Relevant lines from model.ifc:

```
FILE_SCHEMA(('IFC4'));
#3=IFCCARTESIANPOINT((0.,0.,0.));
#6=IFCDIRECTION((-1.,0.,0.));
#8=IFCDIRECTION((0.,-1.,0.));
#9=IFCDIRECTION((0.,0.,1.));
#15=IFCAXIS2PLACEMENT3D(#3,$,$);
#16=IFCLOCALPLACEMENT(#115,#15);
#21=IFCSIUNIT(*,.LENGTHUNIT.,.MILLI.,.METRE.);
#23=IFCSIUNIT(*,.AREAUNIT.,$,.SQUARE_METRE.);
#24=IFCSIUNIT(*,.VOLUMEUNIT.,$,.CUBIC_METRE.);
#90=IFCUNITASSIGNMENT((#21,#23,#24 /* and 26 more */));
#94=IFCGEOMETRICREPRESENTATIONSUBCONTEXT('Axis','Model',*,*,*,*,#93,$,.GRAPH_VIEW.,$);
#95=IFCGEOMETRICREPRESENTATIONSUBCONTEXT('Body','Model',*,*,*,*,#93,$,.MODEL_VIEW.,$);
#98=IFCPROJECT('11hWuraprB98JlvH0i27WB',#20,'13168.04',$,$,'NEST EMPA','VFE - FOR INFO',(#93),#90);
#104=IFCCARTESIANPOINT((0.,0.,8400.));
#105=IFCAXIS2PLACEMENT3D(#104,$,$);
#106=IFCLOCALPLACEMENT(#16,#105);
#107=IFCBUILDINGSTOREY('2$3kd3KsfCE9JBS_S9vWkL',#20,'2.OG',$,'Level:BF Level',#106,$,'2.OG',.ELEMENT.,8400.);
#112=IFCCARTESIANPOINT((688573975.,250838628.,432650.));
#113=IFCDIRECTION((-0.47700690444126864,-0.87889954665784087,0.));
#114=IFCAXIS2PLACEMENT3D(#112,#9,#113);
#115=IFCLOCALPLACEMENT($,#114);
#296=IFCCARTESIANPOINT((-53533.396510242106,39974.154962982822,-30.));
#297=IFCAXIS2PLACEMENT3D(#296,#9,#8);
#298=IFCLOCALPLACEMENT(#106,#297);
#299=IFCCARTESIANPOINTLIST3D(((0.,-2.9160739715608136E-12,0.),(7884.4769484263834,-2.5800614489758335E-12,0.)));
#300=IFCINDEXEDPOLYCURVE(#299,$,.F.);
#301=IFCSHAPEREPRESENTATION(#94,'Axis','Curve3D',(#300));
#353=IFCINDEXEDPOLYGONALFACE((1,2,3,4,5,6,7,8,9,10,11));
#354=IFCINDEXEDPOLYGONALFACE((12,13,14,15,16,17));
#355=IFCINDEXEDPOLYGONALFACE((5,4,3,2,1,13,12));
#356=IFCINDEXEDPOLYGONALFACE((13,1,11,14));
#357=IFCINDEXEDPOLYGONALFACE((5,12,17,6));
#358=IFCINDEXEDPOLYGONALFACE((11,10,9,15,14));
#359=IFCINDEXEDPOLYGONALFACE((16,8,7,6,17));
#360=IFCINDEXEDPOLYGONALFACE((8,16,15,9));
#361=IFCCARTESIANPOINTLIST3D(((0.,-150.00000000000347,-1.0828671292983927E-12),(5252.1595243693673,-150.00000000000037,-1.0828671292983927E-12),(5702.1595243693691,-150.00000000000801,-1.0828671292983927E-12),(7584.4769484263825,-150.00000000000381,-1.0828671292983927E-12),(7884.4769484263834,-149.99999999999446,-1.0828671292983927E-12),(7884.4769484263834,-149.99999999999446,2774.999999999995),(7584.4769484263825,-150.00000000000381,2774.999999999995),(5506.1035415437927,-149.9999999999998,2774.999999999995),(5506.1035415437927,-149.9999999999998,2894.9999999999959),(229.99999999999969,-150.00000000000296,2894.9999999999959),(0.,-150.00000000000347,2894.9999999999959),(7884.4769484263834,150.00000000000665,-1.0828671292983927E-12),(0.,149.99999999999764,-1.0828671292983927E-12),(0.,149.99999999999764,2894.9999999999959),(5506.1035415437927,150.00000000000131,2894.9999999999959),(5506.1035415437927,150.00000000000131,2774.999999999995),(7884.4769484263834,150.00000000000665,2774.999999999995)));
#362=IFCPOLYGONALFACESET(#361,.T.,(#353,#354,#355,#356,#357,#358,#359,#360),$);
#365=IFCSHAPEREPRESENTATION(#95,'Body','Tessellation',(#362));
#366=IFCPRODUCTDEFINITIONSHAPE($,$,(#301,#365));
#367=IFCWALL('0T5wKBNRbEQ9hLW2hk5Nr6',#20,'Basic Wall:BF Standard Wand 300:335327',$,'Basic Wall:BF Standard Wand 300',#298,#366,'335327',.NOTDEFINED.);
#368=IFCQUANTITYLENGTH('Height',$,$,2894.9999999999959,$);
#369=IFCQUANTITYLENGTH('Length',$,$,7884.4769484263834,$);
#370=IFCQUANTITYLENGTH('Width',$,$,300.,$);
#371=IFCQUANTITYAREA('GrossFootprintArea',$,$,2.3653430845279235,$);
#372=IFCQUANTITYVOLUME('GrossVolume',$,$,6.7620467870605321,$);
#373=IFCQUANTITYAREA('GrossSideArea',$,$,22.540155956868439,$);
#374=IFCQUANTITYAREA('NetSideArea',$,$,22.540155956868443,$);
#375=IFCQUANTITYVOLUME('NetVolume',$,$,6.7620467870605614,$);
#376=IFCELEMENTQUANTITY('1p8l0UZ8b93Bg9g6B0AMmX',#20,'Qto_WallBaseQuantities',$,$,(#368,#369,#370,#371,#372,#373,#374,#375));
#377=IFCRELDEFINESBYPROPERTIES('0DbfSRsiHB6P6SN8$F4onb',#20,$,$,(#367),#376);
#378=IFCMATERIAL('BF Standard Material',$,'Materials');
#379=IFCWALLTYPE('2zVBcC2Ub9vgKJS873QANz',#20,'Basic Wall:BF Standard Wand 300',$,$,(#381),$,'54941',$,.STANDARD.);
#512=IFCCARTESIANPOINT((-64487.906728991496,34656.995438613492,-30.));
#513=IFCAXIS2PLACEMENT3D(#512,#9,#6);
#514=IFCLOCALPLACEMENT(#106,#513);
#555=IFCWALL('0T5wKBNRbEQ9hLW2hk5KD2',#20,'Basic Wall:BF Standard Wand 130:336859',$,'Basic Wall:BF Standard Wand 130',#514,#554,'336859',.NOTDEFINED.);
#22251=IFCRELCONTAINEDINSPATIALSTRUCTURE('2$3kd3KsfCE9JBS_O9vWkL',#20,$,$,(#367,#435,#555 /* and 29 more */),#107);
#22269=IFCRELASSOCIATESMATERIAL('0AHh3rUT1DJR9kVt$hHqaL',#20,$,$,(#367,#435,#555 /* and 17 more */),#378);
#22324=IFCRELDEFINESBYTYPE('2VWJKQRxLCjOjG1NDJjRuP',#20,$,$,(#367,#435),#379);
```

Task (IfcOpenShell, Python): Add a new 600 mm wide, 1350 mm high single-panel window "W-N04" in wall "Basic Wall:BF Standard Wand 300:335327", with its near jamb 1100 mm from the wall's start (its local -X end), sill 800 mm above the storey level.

```python
import numpy as np
import ifcopenshell
import ifcopenshell.api.feature
import ifcopenshell.api.geometry
import ifcopenshell.api.pset
import ifcopenshell.api.root
import ifcopenshell.api.spatial
import ifcopenshell.geom
import ifcopenshell.util.element
import ifcopenshell.util.placement
import ifcopenshell.util.representation
import ifcopenshell.util.shape
import ifcopenshell.util.unit

model = ifcopenshell.open("model.ifc")
unit_scale = ifcopenshell.util.unit.calculate_unit_scale(model)
area_scale = ifcopenshell.util.unit.calculate_unit_scale(model, "AREAUNIT")
volume_scale = ifcopenshell.util.unit.calculate_unit_scale(model, "VOLUMEUNIT")
settings = ifcopenshell.geom.settings()


def volume(element):
    """Net volume in cubic metres, openings subtracted."""
    shape = ifcopenshell.geom.create_shape(settings, element)
    return ifcopenshell.util.shape.get_volume(shape.geometry)


wall = model.by_guid("0T5wKBNRbEQ9hLW2hk5Nr6")
storey = ifcopenshell.util.element.get_container(wall, ifc_class="IfcBuildingStorey")
context = ifcopenshell.util.representation.get_context(model, "Model", "Body", "MODEL_VIEW")
before = volume(wall)

width, height, from_end, sill = 0.6, 1.35, 1.1, 0.8  # metres

# The wall runs along its own X axis, and the end named is its -X end.
wall_shape = ifcopenshell.geom.create_shape(settings, wall)
x, y, z = ifcopenshell.util.shape.get_vertices(wall_shape.geometry).T
start = x.min() + from_end
face, thickness = float(y.min()), float(y.max() - y.min())
wall_matrix = ifcopenshell.util.placement.get_local_placement(wall.ObjectPlacement)
level = ifcopenshell.util.placement.get_local_placement(storey.ObjectPlacement)[2, 3]


def in_wall(x, y):
    """Placement at x, y metres in the wall's axes, at sill height."""
    matrix = wall_matrix.copy()
    matrix[:, 3] = wall_matrix @ np.array([x / unit_scale, y / unit_scale, 0.0, 1.0])
    matrix[2, 3] = level + sill / unit_scale
    return matrix


# Opening: a box that overshoots both wall faces by 50 mm.
opening = ifcopenshell.api.root.create_entity(model, ifc_class="IfcOpeningElement", predefined_type="OPENING")
box = ifcopenshell.api.geometry.add_wall_representation(
    model, context=context, length=width, height=height, thickness=thickness + 0.1
)
ifcopenshell.api.geometry.assign_representation(model, product=opening, representation=box)
ifcopenshell.api.geometry.edit_object_placement(model, product=opening, matrix=in_wall(start, face - 0.05), is_si=False)
ifcopenshell.api.feature.add_feature(model, feature=opening, element=wall)

window = ifcopenshell.api.root.create_entity(model, ifc_class="IfcWindow", name="W-N04", predefined_type="WINDOW")
window.OverallWidth, window.OverallHeight = width / unit_scale, height / unit_scale
window.PartitioningType = "SINGLE_PANEL"
body = ifcopenshell.api.geometry.add_window_representation(
    model,
    context=context,
    overall_width=window.OverallWidth,
    overall_height=window.OverallHeight,
    partition_type="SINGLE_PANEL",
)
ifcopenshell.api.geometry.assign_representation(model, product=window, representation=body)
ifcopenshell.api.spatial.assign_container(model, products=[window], relating_structure=storey)
ifcopenshell.api.feature.add_filling(model, opening=opening, element=window)

# Centre the window in the wall's thickness.
ifcopenshell.api.geometry.edit_object_placement(model, product=window, matrix=in_wall(start, face), is_si=False)
window_shape = ifcopenshell.geom.create_shape(settings, window)
depth = ifcopenshell.util.shape.get_vertices(window_shape.geometry)[:, 1]
offset = face + thickness / 2 - (depth.min() + depth.max()) / 2
ifcopenshell.api.geometry.edit_object_placement(model, product=window, matrix=in_wall(start, offset), is_si=False)

after = volume(wall)

# Update the wall's stored quantities.
qto = model.by_id(ifcopenshell.util.element.get_pset(wall, "Qto_WallBaseQuantities", should_inherit=False)["id"])
ifcopenshell.api.pset.edit_qto(model, qto=qto, properties={
    "NetSideArea": after / thickness / area_scale,
    "NetVolume": after / volume_scale,
})

print(f"wall volume {before:.3f} -> {after:.3f} m3")

model.write("model-out.ifc")
```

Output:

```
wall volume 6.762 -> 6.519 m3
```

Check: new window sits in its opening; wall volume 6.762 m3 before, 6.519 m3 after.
